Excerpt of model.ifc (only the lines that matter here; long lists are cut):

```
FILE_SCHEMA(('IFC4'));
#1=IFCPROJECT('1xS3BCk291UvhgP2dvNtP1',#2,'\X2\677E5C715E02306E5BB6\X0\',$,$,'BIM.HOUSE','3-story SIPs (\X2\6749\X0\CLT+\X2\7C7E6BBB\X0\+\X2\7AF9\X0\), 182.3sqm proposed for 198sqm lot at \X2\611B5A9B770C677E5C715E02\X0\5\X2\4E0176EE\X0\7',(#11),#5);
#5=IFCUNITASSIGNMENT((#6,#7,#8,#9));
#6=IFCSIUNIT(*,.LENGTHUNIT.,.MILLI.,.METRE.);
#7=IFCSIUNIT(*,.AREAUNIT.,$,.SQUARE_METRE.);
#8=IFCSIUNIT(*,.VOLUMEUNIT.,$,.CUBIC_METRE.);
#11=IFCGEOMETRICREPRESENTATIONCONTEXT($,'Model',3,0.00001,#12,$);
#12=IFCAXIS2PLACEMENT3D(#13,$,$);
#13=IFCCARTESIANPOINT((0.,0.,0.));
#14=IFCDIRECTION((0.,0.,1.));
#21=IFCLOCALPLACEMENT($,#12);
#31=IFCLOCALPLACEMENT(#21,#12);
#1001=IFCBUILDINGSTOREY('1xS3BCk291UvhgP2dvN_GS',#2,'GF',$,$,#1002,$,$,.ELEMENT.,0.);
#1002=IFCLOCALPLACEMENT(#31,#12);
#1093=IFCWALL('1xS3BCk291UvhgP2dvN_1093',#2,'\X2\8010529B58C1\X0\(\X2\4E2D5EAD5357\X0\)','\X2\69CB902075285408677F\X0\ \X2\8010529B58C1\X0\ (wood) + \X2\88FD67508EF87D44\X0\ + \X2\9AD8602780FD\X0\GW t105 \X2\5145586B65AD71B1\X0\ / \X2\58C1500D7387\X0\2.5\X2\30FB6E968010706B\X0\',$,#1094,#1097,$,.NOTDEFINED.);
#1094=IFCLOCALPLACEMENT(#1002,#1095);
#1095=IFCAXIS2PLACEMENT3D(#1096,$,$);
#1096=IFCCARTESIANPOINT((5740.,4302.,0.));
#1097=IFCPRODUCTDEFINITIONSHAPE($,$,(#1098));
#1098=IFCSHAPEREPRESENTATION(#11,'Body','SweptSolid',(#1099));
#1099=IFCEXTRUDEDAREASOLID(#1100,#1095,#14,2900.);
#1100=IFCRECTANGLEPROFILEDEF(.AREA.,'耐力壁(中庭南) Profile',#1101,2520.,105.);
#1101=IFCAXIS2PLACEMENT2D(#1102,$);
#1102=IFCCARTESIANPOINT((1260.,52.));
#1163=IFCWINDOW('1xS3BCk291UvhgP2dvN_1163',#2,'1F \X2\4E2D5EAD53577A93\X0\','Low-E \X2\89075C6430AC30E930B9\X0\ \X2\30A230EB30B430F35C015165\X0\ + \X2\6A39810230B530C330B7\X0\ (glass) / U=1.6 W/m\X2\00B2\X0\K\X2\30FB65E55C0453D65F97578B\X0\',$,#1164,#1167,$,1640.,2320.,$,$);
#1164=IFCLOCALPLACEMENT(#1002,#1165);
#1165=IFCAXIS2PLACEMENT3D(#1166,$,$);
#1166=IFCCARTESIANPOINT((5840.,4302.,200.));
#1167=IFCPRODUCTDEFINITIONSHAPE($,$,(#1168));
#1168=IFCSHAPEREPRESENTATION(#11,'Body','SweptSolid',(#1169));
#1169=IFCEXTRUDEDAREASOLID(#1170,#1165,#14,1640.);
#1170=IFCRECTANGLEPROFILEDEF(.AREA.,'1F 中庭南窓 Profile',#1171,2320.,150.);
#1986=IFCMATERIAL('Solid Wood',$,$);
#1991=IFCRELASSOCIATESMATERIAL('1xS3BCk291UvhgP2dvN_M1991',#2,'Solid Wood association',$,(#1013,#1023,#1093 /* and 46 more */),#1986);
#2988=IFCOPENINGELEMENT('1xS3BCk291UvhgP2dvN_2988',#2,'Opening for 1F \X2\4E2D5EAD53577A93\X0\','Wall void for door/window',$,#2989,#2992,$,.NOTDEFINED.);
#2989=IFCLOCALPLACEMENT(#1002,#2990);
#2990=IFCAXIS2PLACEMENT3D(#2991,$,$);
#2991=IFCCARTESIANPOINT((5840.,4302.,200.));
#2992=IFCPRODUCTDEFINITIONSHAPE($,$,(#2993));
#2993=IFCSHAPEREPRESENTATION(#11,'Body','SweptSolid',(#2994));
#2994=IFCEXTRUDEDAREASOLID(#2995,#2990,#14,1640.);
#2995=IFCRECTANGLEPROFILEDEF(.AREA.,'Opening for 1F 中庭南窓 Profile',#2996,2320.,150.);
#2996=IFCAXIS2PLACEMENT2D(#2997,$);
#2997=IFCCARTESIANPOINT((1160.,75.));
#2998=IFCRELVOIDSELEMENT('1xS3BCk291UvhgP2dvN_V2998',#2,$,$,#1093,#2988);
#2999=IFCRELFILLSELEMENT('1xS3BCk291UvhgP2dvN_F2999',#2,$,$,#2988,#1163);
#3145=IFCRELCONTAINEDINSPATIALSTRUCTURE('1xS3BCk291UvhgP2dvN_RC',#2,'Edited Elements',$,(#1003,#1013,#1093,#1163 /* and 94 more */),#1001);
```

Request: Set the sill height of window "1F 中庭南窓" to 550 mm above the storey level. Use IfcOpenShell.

```python
import numpy as np
import ifcopenshell
import ifcopenshell.api.geometry
import ifcopenshell.geom
import ifcopenshell.util.element
import ifcopenshell.util.placement
import ifcopenshell.util.shape
import ifcopenshell.util.unit

model = ifcopenshell.open("model.ifc")
unit_scale = ifcopenshell.util.unit.calculate_unit_scale(model)

window = model.by_guid("1xS3BCk291UvhgP2dvN_1163")
opening = window.FillsVoids[0].RelatingOpeningElement
storey = ifcopenshell.util.element.get_container(window, ifc_class="IfcBuildingStorey")
level = ifcopenshell.util.placement.get_local_placement(storey.ObjectPlacement)[2, 3]

# The opening's origin need not be at the sill, so measure its lowest point.
shape = ifcopenshell.geom.create_shape(ifcopenshell.geom.settings(), opening)
bottom = ifcopenshell.util.shape.get_shape_bottom_elevation(shape, shape.geometry) / unit_scale
dz = level + 0.55 / unit_scale - bottom

shift = np.array([0.0, 0.0, dz])
# The window is not placed relative to its opening, so move both.
for product in (opening, window):
    matrix = ifcopenshell.util.placement.get_local_placement(product.ObjectPlacement)
    matrix[:3, 3] += shift
    ifcopenshell.api.geometry.edit_object_placement(model, product=product, matrix=matrix, is_si=False)

print(f"moved by {dz * unit_scale:+.3f} m")

model.write("model_v2.ifc")
```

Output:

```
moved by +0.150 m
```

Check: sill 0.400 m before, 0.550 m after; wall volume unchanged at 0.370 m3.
